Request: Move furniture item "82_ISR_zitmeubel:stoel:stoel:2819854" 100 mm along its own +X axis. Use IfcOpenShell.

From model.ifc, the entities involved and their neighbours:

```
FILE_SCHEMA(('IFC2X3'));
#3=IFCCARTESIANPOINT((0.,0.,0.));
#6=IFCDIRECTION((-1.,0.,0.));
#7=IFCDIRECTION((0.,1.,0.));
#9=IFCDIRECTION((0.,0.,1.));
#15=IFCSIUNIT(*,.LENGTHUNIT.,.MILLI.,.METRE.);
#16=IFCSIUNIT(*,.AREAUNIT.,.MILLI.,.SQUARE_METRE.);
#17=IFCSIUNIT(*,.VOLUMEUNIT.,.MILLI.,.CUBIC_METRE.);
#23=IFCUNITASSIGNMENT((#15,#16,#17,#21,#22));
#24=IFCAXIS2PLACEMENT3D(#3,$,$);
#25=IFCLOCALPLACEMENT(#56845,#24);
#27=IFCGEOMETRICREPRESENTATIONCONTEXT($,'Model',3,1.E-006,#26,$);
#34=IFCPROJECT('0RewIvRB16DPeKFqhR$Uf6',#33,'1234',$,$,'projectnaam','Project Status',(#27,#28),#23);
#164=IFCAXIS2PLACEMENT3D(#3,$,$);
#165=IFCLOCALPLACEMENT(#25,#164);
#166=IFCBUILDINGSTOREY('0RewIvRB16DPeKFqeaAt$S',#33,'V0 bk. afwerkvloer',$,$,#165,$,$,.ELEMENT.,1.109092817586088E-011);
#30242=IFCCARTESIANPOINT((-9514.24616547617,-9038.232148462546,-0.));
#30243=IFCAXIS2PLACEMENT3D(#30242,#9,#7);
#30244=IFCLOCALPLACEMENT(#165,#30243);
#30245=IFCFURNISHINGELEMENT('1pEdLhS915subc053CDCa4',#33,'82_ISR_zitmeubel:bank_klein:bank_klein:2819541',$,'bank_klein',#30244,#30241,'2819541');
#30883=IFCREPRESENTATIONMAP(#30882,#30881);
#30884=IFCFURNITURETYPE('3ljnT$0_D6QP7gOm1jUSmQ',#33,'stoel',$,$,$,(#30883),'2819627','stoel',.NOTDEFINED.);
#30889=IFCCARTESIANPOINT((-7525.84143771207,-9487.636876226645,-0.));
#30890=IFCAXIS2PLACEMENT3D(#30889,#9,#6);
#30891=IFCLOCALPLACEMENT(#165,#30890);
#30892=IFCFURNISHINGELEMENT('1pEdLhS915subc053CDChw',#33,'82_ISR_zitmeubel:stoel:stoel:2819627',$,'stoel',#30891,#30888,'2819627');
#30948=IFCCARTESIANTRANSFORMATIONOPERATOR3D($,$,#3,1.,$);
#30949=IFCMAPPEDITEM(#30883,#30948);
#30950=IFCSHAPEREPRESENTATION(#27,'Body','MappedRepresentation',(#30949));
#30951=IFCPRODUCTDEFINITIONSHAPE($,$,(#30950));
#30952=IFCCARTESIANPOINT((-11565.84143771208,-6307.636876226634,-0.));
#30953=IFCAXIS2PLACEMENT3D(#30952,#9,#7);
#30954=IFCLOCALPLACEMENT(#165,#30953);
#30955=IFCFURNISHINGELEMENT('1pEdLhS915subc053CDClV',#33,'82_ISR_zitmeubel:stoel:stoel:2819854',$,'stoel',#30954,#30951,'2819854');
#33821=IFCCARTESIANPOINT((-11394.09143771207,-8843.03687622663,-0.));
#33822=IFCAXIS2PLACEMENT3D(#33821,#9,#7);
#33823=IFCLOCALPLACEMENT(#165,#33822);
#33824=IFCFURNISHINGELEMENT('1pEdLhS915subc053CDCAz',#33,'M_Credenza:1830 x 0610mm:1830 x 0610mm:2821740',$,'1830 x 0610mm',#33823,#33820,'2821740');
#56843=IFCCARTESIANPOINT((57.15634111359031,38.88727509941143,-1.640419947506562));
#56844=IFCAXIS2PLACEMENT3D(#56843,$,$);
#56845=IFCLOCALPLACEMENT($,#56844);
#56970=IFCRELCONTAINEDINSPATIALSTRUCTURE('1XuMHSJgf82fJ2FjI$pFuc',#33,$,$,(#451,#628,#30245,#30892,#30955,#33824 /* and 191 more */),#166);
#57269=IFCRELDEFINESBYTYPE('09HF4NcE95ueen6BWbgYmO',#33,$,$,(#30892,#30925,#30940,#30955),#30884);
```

```python
import ifcopenshell
import ifcopenshell.api.geometry
import ifcopenshell.util.placement

model = ifcopenshell.open("model.ifc")

item = model.by_guid("1pEdLhS915subc053CDClV")
matrix = ifcopenshell.util.placement.get_local_placement(item.ObjectPlacement)
matrix[:3, 3] += matrix[:3, 0] * 100.0
ifcopenshell.api.geometry.edit_object_placement(model, product=item, matrix=matrix, is_si=False)

print(ifcopenshell.util.placement.get_local_placement(item.ObjectPlacement).round(3) + 0.0)

model.write("model-out.ifc")
```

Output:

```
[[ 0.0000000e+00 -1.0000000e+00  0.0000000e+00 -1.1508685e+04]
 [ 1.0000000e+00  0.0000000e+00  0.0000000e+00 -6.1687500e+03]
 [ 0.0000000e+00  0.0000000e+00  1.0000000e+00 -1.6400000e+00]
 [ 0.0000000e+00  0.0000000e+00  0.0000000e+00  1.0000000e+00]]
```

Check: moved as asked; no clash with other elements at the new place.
